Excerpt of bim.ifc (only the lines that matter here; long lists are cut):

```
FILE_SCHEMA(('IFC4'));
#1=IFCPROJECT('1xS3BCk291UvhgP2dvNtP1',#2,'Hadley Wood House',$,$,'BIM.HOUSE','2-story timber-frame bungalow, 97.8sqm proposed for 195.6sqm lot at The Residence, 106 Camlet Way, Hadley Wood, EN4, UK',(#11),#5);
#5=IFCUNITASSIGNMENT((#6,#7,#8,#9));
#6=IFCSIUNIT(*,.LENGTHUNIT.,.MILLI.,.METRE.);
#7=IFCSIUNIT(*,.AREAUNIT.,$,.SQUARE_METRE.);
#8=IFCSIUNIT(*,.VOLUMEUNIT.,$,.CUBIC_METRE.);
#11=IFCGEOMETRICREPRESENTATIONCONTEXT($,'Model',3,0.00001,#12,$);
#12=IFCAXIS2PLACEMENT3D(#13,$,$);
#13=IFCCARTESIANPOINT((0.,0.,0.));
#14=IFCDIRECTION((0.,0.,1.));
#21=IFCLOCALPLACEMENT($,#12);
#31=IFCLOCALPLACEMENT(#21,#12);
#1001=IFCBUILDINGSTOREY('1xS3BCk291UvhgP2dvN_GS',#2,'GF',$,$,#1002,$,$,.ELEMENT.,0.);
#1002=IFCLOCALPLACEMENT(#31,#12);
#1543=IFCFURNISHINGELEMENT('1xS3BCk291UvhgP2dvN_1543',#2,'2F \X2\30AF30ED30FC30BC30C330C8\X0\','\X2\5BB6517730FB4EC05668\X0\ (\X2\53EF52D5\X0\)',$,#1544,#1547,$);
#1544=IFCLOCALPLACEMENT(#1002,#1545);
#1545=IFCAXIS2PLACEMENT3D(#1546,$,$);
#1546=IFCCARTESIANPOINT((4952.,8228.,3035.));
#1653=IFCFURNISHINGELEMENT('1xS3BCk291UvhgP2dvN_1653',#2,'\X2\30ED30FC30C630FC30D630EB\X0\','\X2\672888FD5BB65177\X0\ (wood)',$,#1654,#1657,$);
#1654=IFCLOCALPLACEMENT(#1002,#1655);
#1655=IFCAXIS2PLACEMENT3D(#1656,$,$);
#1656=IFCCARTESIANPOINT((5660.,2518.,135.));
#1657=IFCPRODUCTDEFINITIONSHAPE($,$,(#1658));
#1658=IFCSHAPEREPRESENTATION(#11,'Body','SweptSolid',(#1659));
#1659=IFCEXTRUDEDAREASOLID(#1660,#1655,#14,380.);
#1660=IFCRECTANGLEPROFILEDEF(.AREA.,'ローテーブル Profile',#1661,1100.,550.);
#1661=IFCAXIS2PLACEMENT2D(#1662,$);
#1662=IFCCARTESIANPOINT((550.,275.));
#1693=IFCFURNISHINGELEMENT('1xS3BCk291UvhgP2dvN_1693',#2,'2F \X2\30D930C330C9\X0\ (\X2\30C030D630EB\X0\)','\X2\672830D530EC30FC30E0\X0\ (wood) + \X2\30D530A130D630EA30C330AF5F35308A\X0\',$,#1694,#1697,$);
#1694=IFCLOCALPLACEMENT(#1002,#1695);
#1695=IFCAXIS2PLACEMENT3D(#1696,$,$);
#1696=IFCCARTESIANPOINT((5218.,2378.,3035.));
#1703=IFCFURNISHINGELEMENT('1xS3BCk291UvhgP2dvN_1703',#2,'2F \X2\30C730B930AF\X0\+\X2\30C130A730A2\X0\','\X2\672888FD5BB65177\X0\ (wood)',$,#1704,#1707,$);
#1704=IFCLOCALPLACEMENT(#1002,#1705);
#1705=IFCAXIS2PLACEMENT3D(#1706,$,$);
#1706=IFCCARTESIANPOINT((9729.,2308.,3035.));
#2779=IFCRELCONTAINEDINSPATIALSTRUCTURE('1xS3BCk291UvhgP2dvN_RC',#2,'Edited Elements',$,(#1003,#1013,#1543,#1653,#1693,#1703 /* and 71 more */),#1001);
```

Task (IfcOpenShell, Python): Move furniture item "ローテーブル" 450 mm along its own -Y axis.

```python
import ifcopenshell
import ifcopenshell.api.geometry
import ifcopenshell.util.placement

model = ifcopenshell.open("bim.ifc")

item = model.by_guid("1xS3BCk291UvhgP2dvN_1653")
matrix = ifcopenshell.util.placement.get_local_placement(item.ObjectPlacement)
matrix[:3, 3] -= matrix[:3, 1] * 450.0
ifcopenshell.api.geometry.edit_object_placement(model, product=item, matrix=matrix, is_si=False)

print(ifcopenshell.util.placement.get_local_placement(item.ObjectPlacement).round(3) + 0.0)

model.write("bim-out.ifc")
```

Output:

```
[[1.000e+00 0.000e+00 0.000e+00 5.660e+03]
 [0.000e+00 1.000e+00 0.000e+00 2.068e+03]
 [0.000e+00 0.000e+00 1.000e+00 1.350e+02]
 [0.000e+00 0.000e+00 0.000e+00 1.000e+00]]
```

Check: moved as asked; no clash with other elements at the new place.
